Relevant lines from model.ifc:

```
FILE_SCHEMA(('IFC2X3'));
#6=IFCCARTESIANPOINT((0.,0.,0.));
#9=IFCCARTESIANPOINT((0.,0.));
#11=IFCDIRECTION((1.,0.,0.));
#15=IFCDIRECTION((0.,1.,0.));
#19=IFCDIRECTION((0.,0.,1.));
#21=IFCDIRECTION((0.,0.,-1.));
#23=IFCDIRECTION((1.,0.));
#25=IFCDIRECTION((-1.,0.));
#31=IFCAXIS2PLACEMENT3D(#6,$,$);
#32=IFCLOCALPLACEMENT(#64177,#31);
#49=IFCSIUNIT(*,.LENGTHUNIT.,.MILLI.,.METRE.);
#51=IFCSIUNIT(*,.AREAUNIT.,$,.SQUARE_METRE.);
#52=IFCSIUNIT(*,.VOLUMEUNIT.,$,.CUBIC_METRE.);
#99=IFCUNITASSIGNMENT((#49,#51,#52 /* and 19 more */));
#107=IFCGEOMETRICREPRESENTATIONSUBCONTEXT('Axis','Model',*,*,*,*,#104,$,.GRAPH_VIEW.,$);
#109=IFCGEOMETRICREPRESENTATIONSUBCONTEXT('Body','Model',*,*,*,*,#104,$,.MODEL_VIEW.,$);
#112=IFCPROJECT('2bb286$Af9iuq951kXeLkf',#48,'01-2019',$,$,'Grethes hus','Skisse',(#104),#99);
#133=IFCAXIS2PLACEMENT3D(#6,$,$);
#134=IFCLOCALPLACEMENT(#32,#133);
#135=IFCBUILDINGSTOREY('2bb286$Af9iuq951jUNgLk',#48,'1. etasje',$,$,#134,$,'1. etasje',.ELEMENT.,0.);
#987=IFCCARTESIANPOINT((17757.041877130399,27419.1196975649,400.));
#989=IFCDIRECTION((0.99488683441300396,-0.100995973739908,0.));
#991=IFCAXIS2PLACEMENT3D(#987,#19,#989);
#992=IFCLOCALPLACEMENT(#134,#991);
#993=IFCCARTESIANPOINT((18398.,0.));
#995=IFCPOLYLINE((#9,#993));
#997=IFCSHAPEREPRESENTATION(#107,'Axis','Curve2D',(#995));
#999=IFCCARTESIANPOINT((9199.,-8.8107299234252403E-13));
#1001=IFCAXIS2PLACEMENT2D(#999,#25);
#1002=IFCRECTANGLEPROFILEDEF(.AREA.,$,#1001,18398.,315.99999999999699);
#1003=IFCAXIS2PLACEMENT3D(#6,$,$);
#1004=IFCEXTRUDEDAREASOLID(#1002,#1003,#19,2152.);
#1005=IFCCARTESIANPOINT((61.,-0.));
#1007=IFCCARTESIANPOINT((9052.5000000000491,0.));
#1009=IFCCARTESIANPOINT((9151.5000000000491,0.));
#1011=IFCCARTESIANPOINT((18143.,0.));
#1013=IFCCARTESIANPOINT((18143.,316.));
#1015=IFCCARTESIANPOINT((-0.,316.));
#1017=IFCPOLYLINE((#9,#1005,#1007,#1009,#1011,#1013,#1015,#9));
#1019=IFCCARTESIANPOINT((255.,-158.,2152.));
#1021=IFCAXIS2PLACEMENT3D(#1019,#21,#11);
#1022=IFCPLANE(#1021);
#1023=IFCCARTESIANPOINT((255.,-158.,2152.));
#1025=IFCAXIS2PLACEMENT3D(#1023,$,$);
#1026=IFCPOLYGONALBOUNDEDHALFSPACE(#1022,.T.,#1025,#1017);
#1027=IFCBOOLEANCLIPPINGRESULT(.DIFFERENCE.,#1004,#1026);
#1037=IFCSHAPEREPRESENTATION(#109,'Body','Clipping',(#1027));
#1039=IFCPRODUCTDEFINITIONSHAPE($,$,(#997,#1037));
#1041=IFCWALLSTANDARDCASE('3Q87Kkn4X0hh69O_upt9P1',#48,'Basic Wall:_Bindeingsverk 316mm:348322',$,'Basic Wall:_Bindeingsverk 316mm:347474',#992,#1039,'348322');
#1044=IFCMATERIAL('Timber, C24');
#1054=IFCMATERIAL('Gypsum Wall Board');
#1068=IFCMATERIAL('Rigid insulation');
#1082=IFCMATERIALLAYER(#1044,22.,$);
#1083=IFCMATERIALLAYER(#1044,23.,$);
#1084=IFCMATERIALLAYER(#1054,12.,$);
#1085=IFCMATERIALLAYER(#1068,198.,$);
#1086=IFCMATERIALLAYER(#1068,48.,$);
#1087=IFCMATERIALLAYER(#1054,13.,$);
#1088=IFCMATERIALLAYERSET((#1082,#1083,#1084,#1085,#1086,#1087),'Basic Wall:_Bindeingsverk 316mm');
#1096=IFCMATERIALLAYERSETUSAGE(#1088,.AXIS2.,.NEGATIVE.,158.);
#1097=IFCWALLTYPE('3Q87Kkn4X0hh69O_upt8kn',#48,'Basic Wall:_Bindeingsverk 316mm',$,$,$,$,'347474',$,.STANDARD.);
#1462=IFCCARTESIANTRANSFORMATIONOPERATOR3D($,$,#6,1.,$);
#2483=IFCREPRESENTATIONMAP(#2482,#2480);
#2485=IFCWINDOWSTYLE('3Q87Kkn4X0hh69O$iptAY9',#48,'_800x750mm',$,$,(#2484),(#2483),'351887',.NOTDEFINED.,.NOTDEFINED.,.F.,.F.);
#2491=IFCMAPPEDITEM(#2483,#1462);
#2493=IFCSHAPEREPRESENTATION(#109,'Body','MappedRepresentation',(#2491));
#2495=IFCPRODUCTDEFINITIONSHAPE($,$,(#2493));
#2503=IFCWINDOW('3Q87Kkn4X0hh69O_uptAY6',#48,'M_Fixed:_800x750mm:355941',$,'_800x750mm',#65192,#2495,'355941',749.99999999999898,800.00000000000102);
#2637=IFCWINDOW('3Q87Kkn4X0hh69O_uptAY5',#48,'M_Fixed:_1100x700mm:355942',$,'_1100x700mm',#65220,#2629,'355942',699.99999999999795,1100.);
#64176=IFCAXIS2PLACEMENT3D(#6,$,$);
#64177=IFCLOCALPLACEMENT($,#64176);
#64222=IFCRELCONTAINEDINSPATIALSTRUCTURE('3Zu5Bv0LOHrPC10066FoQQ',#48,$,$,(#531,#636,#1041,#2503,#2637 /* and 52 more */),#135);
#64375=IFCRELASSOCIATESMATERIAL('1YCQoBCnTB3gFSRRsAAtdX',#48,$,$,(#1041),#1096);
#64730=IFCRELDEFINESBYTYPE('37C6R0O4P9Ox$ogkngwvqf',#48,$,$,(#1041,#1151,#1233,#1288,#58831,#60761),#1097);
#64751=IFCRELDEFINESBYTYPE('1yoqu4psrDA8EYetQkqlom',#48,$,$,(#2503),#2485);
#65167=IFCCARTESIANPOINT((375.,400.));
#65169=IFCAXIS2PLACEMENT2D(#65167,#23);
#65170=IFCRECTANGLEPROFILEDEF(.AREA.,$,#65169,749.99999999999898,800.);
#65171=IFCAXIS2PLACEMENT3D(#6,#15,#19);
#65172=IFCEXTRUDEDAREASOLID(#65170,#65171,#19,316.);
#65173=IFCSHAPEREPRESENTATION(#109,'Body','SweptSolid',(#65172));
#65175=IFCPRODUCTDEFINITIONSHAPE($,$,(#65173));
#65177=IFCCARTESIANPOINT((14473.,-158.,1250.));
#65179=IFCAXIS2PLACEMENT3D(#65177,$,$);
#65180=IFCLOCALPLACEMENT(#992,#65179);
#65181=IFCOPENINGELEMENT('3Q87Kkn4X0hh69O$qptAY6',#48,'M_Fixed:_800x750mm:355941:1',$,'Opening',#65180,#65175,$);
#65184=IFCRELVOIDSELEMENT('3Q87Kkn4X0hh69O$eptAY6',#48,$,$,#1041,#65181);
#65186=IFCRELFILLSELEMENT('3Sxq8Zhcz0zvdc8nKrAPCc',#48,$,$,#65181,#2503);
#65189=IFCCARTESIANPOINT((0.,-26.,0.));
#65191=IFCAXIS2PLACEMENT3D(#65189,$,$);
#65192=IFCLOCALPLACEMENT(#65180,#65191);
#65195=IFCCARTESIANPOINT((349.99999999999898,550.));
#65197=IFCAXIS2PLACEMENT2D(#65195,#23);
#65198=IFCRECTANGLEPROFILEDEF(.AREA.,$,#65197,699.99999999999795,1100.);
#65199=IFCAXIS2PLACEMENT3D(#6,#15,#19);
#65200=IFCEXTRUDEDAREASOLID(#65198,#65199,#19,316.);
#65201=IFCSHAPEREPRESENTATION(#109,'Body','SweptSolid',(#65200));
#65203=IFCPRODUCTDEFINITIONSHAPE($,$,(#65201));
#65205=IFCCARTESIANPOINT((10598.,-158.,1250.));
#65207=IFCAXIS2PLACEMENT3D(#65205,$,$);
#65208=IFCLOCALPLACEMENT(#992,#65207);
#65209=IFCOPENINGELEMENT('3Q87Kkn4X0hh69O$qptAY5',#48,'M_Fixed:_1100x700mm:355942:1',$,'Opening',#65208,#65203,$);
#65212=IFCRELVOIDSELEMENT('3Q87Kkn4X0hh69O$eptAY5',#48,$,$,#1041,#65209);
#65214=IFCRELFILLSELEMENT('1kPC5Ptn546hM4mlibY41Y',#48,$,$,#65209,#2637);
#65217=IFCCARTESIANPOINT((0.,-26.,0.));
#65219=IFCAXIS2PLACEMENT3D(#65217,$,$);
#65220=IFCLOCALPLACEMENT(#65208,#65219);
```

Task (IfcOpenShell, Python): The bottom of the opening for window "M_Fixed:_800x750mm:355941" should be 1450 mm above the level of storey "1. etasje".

```python
import numpy as np
import ifcopenshell
import ifcopenshell.api.geometry
import ifcopenshell.geom
import ifcopenshell.util.element
import ifcopenshell.util.placement
import ifcopenshell.util.shape
import ifcopenshell.util.unit

model = ifcopenshell.open("model.ifc")
unit_scale = ifcopenshell.util.unit.calculate_unit_scale(model)

window = model.by_guid("3Q87Kkn4X0hh69O_uptAY6")
opening = window.FillsVoids[0].RelatingOpeningElement
storey = ifcopenshell.util.element.get_container(window, ifc_class="IfcBuildingStorey")
level = ifcopenshell.util.placement.get_local_placement(storey.ObjectPlacement)[2, 3]

# The opening's origin need not be at the sill, so measure its lowest point.
shape = ifcopenshell.geom.create_shape(ifcopenshell.geom.settings(), opening)
bottom = ifcopenshell.util.shape.get_shape_bottom_elevation(shape, shape.geometry) / unit_scale
dz = level + 1.45 / unit_scale - bottom

shift = np.array([0.0, 0.0, dz])
# The window is placed relative to its opening, so it follows when the opening moves.
matrix = ifcopenshell.util.placement.get_local_placement(opening.ObjectPlacement)
matrix[:3, 3] += shift
ifcopenshell.api.geometry.edit_object_placement(
    model, product=opening, matrix=matrix, is_si=False, should_transform_children=True
)

print(f"moved by {dz * unit_scale:+.3f} m")

model.write("model_edited.ifc")
```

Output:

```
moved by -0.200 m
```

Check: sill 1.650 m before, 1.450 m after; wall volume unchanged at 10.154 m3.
